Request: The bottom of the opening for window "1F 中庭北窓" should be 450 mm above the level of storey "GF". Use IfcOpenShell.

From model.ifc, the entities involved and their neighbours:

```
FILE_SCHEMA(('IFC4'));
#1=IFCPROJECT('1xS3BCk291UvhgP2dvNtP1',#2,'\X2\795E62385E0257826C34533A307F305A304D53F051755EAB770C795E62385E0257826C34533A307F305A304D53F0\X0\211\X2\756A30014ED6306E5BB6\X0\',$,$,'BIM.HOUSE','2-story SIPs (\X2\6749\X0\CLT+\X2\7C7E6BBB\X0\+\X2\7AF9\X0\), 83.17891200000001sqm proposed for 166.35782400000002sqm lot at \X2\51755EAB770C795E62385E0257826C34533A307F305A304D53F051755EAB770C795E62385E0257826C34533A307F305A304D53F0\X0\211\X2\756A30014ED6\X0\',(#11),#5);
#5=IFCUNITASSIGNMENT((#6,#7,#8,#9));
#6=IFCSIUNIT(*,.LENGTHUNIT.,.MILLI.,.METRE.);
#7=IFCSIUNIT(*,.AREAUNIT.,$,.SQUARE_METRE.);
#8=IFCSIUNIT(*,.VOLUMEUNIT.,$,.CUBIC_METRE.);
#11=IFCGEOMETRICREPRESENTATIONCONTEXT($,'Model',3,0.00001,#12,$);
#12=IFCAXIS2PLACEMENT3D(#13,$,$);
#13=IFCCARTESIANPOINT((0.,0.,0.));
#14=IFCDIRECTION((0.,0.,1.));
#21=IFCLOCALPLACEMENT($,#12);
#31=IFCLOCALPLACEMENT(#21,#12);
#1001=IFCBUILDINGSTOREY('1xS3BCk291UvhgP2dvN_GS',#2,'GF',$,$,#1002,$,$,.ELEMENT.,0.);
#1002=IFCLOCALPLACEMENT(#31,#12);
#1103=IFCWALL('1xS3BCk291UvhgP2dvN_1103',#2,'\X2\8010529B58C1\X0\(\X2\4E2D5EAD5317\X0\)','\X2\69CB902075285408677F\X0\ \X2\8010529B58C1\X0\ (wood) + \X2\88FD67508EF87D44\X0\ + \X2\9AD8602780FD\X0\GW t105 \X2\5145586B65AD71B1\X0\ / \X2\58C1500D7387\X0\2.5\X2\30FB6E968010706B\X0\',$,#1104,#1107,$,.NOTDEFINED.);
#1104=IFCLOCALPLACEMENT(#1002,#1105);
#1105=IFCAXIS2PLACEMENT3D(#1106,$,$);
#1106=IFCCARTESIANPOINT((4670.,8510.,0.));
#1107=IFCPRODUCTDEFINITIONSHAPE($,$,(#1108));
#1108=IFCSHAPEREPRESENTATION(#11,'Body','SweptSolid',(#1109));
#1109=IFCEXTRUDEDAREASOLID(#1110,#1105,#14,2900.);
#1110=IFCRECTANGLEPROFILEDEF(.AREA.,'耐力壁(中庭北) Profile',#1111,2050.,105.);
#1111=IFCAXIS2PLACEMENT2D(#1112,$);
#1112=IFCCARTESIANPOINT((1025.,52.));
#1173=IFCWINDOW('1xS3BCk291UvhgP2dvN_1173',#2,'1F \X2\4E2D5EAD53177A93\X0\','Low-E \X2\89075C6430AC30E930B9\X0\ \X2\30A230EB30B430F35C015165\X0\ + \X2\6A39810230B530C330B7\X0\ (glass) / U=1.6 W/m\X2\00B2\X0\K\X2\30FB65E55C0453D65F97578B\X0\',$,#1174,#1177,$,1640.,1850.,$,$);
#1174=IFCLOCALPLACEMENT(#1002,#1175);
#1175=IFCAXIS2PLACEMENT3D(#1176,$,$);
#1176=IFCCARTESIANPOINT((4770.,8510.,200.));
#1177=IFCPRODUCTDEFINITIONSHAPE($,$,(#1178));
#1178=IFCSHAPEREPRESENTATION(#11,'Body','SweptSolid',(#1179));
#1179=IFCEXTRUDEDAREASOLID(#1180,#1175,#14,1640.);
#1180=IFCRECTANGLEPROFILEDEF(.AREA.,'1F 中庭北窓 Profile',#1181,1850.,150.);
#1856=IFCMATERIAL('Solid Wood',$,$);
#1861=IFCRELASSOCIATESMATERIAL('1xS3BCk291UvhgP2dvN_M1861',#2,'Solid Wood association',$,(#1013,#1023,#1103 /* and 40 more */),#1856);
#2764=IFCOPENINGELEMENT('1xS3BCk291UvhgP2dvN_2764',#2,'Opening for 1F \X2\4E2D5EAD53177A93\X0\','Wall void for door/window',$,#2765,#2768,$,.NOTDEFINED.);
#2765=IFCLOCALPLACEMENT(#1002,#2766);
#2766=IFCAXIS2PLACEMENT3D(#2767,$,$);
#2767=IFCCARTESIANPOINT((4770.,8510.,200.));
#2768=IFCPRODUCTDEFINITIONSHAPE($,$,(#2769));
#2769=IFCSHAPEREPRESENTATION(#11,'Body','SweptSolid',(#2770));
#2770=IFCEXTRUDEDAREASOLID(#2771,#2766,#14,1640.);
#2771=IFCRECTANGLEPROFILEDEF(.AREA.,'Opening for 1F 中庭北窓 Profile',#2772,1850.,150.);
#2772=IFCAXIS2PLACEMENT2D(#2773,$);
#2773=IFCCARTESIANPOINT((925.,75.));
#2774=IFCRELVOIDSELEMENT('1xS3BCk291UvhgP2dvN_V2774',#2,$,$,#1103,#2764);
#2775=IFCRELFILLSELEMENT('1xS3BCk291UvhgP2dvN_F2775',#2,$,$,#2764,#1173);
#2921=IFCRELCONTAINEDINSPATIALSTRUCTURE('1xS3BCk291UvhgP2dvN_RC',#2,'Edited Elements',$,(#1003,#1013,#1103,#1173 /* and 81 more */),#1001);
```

```python
import numpy as np
import ifcopenshell
import ifcopenshell.api.geometry
import ifcopenshell.geom
import ifcopenshell.util.element
import ifcopenshell.util.placement
import ifcopenshell.util.shape
import ifcopenshell.util.unit

model = ifcopenshell.open("model.ifc")
unit_scale = ifcopenshell.util.unit.calculate_unit_scale(model)

window = model.by_id(1173)
opening = window.FillsVoids[0].RelatingOpeningElement
storey = ifcopenshell.util.element.get_container(window, ifc_class="IfcBuildingStorey")
level = ifcopenshell.util.placement.get_local_placement(storey.ObjectPlacement)[2, 3]

# The opening's origin need not be at the sill, so measure its lowest point.
shape = ifcopenshell.geom.create_shape(ifcopenshell.geom.settings(), opening)
bottom = ifcopenshell.util.shape.get_shape_bottom_elevation(shape, shape.geometry) / unit_scale
dz = level + 0.45 / unit_scale - bottom

shift = np.array([0.0, 0.0, dz])
# The window is not placed relative to its opening, so move both.
for product in (opening, window):
    matrix = ifcopenshell.util.placement.get_local_placement(product.ObjectPlacement)
    matrix[:3, 3] += shift
    ifcopenshell.api.geometry.edit_object_placement(model, product=product, matrix=matrix, is_si=False)

print(f"moved by {dz * unit_scale:+.3f} m")

model.write("model_updated.ifc")
```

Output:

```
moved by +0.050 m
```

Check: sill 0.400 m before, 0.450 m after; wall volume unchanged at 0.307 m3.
